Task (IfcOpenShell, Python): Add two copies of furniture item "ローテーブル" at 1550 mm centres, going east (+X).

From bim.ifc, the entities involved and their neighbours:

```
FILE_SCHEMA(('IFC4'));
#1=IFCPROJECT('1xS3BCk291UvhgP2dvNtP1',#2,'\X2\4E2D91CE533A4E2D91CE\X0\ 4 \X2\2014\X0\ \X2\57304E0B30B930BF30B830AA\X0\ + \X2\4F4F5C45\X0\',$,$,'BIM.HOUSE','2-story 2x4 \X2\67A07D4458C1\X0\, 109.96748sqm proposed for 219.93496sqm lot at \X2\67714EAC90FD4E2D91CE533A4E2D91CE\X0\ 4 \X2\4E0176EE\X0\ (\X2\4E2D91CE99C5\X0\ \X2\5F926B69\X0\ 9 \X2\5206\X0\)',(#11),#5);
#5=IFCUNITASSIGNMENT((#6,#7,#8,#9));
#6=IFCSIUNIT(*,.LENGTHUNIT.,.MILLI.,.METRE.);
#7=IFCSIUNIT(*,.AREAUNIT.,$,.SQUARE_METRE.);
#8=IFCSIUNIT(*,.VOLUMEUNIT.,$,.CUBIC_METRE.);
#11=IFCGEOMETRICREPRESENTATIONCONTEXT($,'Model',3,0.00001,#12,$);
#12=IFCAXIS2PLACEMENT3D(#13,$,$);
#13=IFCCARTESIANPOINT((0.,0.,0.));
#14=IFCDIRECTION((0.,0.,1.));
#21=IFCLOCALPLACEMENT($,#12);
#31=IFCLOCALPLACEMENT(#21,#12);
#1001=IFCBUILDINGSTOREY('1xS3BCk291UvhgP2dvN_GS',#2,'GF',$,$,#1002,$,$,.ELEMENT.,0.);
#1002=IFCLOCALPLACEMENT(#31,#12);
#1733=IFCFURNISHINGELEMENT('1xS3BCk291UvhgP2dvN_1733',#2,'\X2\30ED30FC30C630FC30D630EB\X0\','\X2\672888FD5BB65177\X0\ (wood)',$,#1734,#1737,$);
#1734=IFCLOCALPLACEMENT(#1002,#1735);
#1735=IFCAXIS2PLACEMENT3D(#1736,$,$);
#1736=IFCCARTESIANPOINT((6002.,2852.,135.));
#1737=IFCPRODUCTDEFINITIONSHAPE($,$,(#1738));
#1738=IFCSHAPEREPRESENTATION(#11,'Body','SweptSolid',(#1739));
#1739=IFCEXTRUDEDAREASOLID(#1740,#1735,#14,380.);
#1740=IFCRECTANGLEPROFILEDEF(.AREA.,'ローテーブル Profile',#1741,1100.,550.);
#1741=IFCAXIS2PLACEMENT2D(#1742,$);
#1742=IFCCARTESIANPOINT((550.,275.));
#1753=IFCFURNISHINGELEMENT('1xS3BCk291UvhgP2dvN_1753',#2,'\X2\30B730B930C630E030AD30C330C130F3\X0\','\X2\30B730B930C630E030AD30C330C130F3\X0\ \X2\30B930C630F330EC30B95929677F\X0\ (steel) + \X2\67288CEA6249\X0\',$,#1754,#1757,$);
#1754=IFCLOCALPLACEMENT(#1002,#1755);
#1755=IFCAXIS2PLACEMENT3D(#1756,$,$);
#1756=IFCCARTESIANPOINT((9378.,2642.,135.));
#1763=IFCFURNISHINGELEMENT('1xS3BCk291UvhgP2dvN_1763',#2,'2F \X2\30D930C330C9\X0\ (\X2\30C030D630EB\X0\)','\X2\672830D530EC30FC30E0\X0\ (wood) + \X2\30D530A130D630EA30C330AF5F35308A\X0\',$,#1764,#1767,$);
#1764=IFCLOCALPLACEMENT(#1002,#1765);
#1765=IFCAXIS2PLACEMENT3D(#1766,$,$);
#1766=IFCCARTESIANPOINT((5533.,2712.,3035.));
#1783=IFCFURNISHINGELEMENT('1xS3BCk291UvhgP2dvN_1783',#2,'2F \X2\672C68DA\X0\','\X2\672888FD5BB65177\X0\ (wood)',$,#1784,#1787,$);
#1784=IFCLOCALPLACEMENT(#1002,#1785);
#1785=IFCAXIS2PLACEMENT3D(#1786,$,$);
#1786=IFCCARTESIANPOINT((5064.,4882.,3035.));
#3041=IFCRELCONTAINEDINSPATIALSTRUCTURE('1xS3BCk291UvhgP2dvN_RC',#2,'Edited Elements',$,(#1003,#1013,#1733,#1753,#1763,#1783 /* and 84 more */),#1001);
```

```python
import numpy as np
import ifcopenshell
import ifcopenshell.api.geometry
import ifcopenshell.api.root
import ifcopenshell.util.element
import ifcopenshell.util.placement
import ifcopenshell.util.unit

model = ifcopenshell.open("bim.ifc")
unit_scale = ifcopenshell.util.unit.calculate_unit_scale(model)


def reuse_history(source, copy):
    """copy_class also copies each property set's owner history, people and application; keep the originals."""
    for rel in copy.IsDefinedBy:
        if rel.is_a("IfcRelDefinesByProperties") and (history := rel.RelatingPropertyDefinition.OwnerHistory):
            rel.RelatingPropertyDefinition.OwnerHistory = source.OwnerHistory
            ifcopenshell.util.element.remove_deep2(model, history)


source = model.by_guid("1xS3BCk291UvhgP2dvN_1733")
base = ifcopenshell.util.placement.get_local_placement(source.ObjectPlacement)
step = np.array([1.0, 0.0, 0.0]) * 1.55 / unit_scale

for i in range(1, 3):
    copy = ifcopenshell.api.root.copy_class(model, product=source)
    copy.Representation = ifcopenshell.util.element.copy_deep(
        model, source.Representation, exclude=["IfcGeometricRepresentationContext", "IfcRepresentationMap"]
    )
    reuse_history(source, copy)
    matrix = base.copy()
    matrix[:3, 3] += i * step
    print("added at", matrix[:3, 3].round(3) + 0.0)
    ifcopenshell.api.geometry.edit_object_placement(model, product=copy, matrix=matrix, is_si=False)

model.write("bim_v2.ifc")
```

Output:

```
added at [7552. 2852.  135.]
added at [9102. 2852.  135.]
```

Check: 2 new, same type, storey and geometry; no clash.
